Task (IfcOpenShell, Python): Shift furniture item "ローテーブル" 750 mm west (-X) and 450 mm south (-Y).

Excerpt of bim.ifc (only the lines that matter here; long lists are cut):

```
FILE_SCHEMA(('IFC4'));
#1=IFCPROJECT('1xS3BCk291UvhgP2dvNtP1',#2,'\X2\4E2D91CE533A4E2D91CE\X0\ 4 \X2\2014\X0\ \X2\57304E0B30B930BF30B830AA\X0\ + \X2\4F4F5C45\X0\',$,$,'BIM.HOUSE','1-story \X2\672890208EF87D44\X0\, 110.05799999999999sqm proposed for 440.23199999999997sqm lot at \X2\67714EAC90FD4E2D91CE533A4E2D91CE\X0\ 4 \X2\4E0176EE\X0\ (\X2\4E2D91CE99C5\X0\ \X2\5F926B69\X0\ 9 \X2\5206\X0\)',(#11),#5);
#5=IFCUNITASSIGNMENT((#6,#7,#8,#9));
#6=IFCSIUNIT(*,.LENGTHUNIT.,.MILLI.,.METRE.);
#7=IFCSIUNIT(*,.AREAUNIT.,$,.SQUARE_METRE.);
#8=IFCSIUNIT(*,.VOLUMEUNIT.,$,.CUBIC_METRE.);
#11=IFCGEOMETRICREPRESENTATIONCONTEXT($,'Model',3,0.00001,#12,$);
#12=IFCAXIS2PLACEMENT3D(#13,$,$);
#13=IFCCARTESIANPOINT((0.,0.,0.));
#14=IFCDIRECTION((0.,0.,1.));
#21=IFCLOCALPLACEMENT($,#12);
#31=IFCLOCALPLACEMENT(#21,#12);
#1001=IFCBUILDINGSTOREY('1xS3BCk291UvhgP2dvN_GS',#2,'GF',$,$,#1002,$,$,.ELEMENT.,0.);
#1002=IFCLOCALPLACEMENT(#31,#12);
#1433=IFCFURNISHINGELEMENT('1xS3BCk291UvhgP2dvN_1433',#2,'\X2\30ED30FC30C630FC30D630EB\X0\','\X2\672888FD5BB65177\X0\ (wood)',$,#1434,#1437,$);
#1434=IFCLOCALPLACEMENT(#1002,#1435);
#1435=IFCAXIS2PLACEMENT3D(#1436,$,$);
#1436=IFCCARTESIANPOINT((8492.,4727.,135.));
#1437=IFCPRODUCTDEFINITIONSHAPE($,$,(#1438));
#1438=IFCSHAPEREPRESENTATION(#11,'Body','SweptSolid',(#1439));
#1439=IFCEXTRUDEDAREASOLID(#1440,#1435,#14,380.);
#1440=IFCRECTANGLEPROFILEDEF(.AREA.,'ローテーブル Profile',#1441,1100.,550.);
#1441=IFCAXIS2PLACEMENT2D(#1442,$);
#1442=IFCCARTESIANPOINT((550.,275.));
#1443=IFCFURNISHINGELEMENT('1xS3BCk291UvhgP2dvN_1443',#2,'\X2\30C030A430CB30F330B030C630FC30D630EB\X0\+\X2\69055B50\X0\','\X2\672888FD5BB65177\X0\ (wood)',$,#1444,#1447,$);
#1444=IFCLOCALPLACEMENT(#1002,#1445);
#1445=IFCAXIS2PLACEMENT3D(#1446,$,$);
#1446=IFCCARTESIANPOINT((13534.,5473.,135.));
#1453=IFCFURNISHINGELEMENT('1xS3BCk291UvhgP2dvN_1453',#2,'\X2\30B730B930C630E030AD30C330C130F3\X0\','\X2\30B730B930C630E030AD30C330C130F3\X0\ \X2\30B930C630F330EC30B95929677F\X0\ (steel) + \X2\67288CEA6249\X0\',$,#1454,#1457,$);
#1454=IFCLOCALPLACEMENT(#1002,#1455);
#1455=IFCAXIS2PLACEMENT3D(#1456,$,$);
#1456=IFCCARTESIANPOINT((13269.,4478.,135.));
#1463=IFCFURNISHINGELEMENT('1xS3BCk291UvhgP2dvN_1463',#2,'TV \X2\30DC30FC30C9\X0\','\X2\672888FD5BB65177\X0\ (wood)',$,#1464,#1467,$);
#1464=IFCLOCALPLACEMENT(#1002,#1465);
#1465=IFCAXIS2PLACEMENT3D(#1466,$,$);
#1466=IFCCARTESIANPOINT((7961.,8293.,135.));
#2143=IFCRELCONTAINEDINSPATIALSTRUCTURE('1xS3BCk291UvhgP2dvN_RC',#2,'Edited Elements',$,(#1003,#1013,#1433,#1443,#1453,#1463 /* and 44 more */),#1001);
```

```python
import ifcopenshell
import ifcopenshell.api.geometry
import ifcopenshell.util.placement

model = ifcopenshell.open("bim.ifc")

item = model.by_guid("1xS3BCk291UvhgP2dvN_1433")
matrix = ifcopenshell.util.placement.get_local_placement(item.ObjectPlacement)
matrix[0, 3] -= 750.0
matrix[1, 3] -= 450.0
ifcopenshell.api.geometry.edit_object_placement(model, product=item, matrix=matrix, is_si=False)

print(ifcopenshell.util.placement.get_local_placement(item.ObjectPlacement).round(3) + 0.0)

model.write("bim_rev.ifc")
```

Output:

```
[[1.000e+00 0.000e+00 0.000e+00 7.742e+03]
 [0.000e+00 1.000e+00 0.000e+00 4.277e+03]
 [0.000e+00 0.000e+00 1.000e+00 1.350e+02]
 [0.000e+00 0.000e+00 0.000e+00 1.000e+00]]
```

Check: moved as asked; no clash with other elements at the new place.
